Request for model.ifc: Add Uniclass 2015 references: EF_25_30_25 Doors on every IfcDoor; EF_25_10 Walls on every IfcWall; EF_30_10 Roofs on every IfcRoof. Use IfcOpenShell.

First a look at what the model holds.

```python
import ifcopenshell

model = ifcopenshell.open("model.ifc")
print(model.schema)
print("classifications:", [c.Name for c in model.by_type("IfcClassification")])
for ifc_class in ("IfcDoor", "IfcRoof", "IfcStair", "IfcWall", "IfcWindow"):
    print(ifc_class, len(model.by_type(ifc_class)))
```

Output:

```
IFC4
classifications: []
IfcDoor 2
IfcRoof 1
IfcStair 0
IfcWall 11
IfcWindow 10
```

```python
import ifcopenshell
import ifcopenshell.api.classification

model = ifcopenshell.open("model.ifc")

system = ifcopenshell.api.classification.add_classification(model, classification="Uniclass 2015")

codes = {
    "IfcDoor": ("EF_25_30_25", "Doors"),
    "IfcWall": ("EF_25_10", "Walls"),
    "IfcRoof": ("EF_30_10", "Roofs"),
}
for ifc_class, (code, name) in codes.items():
    products = model.by_type(ifc_class)
    ifcopenshell.api.classification.add_reference(
        model, products=products, classification=system, identification=code, name=name
    )
    print(code, len(products))

model.write("model_rev.ifc")
```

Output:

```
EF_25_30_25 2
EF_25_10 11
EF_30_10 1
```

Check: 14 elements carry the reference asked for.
